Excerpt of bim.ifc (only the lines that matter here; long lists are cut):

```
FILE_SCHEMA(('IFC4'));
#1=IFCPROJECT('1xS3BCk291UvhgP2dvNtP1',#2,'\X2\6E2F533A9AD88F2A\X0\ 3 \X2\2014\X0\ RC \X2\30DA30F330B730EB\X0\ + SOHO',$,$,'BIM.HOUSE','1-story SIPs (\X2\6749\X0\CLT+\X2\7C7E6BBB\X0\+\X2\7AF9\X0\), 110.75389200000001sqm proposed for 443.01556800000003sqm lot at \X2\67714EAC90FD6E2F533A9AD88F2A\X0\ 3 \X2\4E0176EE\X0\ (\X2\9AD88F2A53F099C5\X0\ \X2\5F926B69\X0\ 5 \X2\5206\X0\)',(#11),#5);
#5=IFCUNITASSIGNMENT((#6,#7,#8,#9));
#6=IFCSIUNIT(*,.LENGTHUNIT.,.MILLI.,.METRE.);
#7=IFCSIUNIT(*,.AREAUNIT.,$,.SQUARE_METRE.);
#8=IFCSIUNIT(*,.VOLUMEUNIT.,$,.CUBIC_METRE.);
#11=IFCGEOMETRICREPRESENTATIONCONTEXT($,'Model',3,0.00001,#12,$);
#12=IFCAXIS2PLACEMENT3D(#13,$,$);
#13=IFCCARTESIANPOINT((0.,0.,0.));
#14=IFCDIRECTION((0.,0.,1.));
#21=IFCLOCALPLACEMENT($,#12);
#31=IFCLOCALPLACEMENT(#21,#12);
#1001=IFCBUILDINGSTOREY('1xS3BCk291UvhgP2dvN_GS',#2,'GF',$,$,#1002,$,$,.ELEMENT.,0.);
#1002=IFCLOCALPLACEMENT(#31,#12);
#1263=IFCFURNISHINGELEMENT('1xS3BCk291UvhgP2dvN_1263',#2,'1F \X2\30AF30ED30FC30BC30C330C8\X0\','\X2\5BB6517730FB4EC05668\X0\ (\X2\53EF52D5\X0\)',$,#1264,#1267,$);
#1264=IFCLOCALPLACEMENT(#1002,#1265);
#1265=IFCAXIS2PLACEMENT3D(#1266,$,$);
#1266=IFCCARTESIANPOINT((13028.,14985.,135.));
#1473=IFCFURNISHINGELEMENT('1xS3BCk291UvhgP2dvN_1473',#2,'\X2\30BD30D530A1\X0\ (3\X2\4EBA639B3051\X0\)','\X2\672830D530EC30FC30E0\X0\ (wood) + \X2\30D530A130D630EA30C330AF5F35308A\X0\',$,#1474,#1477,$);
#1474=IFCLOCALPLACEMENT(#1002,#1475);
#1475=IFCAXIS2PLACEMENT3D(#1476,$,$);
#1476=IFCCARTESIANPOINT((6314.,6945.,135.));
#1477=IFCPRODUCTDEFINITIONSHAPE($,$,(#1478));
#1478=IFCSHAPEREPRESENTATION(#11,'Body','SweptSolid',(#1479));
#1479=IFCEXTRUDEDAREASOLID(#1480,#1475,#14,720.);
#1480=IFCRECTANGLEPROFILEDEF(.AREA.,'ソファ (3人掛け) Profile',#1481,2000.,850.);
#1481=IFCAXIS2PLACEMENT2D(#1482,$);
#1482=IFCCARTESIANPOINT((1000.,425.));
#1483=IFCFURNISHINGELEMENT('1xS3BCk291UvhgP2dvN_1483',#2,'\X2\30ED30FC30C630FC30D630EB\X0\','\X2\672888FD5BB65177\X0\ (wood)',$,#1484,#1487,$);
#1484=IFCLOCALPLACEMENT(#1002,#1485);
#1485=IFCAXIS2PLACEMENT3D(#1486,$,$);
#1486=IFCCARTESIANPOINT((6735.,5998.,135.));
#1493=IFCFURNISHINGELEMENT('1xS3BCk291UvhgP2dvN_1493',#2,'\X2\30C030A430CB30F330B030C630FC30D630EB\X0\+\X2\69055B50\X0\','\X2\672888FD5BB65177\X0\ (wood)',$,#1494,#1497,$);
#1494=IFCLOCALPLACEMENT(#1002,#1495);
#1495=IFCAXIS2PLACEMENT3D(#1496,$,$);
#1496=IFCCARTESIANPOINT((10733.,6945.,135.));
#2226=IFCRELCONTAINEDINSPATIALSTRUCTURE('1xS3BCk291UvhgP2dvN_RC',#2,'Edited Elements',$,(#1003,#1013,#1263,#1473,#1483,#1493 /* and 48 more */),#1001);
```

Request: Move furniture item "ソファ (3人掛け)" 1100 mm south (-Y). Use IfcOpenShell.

```python
import ifcopenshell
import ifcopenshell.api.geometry
import ifcopenshell.util.placement
import ifcopenshell.util.unit

model = ifcopenshell.open("bim.ifc")
unit_scale = ifcopenshell.util.unit.calculate_unit_scale(model)

item = model.by_id(1473)
matrix = ifcopenshell.util.placement.get_local_placement(item.ObjectPlacement)
matrix[1, 3] -= 1.1 / unit_scale
ifcopenshell.api.geometry.edit_object_placement(model, product=item, matrix=matrix, is_si=False)

print(ifcopenshell.util.placement.get_local_placement(item.ObjectPlacement).round(3) + 0.0)

model.write("bim_v2.ifc")
```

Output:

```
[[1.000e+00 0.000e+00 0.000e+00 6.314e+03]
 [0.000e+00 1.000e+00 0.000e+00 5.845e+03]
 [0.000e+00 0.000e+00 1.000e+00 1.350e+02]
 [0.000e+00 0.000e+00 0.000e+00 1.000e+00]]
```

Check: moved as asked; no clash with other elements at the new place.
